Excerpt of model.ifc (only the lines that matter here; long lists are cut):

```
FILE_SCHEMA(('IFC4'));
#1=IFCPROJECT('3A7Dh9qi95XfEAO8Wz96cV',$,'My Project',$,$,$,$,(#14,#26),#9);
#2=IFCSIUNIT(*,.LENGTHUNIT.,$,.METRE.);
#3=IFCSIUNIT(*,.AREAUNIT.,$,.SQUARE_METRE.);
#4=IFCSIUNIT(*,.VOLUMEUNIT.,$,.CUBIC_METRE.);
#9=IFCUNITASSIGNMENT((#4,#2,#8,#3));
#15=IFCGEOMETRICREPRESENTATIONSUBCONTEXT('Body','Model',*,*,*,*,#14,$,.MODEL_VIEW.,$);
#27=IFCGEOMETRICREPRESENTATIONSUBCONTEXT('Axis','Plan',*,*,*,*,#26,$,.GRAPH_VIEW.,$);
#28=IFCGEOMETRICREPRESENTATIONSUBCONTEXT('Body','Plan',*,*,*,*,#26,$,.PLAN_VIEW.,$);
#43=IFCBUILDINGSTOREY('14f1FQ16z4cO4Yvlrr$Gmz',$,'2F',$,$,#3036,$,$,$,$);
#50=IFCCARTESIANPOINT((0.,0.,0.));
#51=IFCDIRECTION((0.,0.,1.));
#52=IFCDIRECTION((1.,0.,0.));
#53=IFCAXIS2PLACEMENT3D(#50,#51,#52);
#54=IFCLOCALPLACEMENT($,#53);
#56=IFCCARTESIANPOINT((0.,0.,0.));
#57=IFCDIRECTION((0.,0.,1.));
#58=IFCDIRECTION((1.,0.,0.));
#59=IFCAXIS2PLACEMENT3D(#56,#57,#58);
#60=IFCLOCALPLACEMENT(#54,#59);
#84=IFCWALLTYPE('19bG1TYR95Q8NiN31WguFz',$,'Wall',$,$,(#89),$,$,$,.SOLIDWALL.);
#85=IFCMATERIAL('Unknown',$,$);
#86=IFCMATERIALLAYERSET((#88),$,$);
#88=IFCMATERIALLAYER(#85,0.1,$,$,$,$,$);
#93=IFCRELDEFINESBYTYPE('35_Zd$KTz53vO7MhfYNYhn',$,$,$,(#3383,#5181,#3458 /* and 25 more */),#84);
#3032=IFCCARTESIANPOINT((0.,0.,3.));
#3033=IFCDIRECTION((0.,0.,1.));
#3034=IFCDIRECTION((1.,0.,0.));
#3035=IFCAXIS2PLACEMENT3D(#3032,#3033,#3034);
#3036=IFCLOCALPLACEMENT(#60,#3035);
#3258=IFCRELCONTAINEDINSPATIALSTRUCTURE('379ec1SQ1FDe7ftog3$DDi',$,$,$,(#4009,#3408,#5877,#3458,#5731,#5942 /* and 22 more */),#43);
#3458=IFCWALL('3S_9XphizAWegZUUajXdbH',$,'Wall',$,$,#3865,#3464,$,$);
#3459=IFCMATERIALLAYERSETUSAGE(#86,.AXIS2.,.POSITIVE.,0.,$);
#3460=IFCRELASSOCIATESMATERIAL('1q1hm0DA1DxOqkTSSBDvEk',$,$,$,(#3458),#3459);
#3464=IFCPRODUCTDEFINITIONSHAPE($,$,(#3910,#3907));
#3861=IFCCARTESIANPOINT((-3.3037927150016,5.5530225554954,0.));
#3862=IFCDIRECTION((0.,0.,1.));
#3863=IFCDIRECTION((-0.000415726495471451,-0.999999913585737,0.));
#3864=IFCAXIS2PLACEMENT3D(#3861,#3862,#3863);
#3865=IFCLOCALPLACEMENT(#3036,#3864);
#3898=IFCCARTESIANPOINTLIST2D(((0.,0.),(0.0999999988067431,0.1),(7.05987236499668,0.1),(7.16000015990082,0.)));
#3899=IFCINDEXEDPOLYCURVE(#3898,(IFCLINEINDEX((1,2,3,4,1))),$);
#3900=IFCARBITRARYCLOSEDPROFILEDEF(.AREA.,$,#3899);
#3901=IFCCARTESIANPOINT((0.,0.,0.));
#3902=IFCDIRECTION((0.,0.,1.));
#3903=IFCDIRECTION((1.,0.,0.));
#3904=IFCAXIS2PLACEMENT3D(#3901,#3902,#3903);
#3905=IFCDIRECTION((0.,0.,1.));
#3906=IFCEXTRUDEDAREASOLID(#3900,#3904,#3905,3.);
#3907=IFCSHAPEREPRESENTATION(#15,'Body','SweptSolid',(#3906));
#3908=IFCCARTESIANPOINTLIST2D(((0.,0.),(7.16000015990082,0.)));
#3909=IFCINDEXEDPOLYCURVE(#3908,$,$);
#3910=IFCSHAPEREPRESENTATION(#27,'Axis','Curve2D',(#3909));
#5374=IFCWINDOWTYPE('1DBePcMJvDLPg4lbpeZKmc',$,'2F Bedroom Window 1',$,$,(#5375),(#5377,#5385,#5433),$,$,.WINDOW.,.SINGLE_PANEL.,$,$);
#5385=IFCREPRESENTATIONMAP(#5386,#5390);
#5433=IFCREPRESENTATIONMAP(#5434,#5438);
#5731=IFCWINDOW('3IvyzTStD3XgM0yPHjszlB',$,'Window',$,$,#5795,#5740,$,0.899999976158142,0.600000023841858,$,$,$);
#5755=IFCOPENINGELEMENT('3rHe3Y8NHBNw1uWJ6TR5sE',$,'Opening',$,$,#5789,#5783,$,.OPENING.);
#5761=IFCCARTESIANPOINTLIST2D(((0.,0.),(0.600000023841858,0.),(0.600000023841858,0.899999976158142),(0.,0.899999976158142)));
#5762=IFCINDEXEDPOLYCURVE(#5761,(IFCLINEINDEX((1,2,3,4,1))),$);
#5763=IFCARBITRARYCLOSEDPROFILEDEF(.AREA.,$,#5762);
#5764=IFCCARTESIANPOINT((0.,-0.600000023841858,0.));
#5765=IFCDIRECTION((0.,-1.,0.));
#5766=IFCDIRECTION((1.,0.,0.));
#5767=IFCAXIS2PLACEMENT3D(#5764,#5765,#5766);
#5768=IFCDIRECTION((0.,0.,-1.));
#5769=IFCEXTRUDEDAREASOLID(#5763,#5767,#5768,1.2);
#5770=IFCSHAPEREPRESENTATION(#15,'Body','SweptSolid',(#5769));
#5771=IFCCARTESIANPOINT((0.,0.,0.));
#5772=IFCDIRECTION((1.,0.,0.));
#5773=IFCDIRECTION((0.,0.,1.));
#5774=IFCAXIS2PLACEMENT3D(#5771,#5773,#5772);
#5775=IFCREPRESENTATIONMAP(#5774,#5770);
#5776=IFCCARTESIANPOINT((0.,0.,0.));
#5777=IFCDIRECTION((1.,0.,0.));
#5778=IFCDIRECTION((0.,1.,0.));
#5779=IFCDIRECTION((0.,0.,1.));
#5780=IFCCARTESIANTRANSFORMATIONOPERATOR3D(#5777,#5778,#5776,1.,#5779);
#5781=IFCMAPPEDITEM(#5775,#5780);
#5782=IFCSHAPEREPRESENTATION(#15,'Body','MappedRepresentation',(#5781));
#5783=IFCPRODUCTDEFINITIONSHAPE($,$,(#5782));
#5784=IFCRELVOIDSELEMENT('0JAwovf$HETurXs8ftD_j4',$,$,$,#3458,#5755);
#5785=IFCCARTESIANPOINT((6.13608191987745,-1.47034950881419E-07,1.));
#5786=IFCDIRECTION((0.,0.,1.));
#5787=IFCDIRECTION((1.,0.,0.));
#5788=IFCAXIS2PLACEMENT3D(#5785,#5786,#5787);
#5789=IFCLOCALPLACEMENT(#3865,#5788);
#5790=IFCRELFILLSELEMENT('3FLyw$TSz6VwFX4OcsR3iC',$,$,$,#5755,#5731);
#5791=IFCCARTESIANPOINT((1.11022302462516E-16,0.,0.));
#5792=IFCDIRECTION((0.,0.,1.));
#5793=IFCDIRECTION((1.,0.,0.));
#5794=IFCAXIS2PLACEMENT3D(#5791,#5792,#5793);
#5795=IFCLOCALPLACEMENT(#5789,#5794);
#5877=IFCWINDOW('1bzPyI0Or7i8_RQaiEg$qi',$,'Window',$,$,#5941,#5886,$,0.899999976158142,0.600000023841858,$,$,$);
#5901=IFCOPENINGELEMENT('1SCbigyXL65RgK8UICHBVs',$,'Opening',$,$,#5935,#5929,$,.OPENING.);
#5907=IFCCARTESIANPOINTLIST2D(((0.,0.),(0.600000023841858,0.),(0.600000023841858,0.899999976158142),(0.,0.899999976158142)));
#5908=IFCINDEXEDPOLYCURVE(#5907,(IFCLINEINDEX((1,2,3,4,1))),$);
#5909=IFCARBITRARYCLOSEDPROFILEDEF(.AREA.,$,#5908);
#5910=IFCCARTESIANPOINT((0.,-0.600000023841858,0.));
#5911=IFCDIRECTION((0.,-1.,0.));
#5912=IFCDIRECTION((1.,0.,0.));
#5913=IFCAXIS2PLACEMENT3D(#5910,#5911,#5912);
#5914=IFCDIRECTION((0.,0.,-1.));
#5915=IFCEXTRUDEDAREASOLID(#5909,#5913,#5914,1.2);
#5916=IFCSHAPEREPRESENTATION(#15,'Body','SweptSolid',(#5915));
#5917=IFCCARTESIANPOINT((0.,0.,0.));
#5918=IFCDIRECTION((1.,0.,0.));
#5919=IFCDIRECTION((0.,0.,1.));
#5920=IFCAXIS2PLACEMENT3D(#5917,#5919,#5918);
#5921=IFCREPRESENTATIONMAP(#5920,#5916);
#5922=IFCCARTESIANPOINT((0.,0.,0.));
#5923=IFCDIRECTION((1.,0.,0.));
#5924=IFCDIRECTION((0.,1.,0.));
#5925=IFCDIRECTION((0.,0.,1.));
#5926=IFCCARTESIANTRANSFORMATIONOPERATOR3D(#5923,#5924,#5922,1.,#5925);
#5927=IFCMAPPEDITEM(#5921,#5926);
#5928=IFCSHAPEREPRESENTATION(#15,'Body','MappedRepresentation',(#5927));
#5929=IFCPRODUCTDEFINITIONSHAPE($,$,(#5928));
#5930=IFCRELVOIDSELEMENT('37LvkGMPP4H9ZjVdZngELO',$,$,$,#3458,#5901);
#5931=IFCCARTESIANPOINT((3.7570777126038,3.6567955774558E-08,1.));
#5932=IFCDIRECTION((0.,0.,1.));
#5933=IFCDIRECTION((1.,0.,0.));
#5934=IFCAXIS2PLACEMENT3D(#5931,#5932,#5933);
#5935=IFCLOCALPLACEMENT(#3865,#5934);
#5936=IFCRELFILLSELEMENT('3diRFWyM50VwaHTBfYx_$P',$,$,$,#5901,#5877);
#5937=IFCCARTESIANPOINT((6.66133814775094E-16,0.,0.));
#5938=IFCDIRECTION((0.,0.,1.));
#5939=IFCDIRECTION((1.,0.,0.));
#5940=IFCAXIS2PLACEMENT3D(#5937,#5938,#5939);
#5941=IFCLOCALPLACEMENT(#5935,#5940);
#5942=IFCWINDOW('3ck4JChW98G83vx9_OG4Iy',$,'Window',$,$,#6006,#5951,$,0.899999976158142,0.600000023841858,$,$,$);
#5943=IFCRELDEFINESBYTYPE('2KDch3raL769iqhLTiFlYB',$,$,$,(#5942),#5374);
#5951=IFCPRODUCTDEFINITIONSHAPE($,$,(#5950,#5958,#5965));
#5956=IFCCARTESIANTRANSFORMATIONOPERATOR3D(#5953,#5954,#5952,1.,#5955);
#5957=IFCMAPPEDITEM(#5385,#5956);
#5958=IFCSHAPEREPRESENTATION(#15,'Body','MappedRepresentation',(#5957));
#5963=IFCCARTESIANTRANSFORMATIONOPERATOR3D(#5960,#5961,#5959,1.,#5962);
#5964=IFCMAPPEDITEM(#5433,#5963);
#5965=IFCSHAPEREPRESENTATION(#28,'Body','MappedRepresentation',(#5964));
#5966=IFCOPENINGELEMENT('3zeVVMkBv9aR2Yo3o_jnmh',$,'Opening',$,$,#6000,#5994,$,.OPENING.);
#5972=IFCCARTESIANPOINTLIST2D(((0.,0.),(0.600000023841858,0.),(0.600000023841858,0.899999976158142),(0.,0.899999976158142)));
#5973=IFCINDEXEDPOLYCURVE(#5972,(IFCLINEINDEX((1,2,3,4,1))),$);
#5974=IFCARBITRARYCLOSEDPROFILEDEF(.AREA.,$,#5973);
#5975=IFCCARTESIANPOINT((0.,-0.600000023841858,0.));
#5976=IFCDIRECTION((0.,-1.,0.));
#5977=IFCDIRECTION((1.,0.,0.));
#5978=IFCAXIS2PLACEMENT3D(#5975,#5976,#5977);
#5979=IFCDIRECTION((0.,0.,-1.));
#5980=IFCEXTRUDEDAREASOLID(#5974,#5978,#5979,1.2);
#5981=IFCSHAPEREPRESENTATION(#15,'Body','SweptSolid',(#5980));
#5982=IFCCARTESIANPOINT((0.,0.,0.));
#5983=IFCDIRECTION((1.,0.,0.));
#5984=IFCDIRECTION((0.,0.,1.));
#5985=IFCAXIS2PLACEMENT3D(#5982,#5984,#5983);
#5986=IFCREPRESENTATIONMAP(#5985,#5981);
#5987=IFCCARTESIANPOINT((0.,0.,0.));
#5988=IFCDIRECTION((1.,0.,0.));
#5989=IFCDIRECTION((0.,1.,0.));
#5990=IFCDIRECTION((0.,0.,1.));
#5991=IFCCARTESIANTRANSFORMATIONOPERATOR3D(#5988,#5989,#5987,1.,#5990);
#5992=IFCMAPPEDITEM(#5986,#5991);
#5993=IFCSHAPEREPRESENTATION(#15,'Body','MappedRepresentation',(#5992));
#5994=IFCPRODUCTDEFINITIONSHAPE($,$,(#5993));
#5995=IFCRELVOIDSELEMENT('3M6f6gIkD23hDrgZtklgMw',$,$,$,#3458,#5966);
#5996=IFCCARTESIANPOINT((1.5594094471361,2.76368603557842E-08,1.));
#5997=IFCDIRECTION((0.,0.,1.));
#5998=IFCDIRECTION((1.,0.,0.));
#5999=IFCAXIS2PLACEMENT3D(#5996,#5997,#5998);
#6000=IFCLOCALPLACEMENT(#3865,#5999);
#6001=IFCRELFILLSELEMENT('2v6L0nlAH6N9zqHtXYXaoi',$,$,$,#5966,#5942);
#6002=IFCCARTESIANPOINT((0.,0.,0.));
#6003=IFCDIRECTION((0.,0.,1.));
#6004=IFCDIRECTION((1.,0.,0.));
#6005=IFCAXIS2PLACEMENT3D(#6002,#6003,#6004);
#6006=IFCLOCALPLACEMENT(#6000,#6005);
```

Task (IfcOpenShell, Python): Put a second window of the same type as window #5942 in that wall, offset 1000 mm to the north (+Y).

```python
import ifcopenshell
import ifcopenshell.api.feature
import ifcopenshell.api.geometry
import ifcopenshell.api.root
import ifcopenshell.geom
import ifcopenshell.util.element
import ifcopenshell.util.placement
import ifcopenshell.util.shape
import ifcopenshell.util.unit

model = ifcopenshell.open("model.ifc")
unit_scale = ifcopenshell.util.unit.calculate_unit_scale(model)
settings = ifcopenshell.geom.settings()


def volume(element):
    """Net volume in cubic metres, openings subtracted."""
    shape = ifcopenshell.geom.create_shape(settings, element)
    return ifcopenshell.util.shape.get_volume(shape.geometry)


window = model.by_guid("3ck4JChW98G83vx9_OG4Iy")
opening = window.FillsVoids[0].RelatingOpeningElement
wall = opening.VoidsElements[0].RelatingBuildingElement
before = volume(wall)
shift = ifcopenshell.util.placement.get_local_placement(wall.ObjectPlacement)[:3, 0] * -1 / unit_scale

# copy_class copies the void relationship, type, container and properties, but no geometry.
new_opening = ifcopenshell.api.root.copy_class(model, product=opening)
new_opening.Representation = ifcopenshell.util.element.copy_deep(
    model, opening.Representation, exclude=["IfcGeometricRepresentationContext", "IfcRepresentationMap"]
)
new_window = ifcopenshell.api.root.copy_class(model, product=window)
new_window.Representation = ifcopenshell.util.element.copy_deep(
    model, window.Representation, exclude=["IfcGeometricRepresentationContext", "IfcRepresentationMap"]
)
ifcopenshell.api.feature.add_filling(model, opening=new_opening, element=new_window)

for old, new in ((opening, new_opening), (window, new_window)):
    matrix = ifcopenshell.util.placement.get_local_placement(old.ObjectPlacement)
    matrix[:3, 3] += shift
    ifcopenshell.api.geometry.edit_object_placement(model, product=new, matrix=matrix, is_si=False)

after = volume(wall)

print(f"wall volume {before:.3f} -> {after:.3f} m3")

model.write("model_edited.ifc")
```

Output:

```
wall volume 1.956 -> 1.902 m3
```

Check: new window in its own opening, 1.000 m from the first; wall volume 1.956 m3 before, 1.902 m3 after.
